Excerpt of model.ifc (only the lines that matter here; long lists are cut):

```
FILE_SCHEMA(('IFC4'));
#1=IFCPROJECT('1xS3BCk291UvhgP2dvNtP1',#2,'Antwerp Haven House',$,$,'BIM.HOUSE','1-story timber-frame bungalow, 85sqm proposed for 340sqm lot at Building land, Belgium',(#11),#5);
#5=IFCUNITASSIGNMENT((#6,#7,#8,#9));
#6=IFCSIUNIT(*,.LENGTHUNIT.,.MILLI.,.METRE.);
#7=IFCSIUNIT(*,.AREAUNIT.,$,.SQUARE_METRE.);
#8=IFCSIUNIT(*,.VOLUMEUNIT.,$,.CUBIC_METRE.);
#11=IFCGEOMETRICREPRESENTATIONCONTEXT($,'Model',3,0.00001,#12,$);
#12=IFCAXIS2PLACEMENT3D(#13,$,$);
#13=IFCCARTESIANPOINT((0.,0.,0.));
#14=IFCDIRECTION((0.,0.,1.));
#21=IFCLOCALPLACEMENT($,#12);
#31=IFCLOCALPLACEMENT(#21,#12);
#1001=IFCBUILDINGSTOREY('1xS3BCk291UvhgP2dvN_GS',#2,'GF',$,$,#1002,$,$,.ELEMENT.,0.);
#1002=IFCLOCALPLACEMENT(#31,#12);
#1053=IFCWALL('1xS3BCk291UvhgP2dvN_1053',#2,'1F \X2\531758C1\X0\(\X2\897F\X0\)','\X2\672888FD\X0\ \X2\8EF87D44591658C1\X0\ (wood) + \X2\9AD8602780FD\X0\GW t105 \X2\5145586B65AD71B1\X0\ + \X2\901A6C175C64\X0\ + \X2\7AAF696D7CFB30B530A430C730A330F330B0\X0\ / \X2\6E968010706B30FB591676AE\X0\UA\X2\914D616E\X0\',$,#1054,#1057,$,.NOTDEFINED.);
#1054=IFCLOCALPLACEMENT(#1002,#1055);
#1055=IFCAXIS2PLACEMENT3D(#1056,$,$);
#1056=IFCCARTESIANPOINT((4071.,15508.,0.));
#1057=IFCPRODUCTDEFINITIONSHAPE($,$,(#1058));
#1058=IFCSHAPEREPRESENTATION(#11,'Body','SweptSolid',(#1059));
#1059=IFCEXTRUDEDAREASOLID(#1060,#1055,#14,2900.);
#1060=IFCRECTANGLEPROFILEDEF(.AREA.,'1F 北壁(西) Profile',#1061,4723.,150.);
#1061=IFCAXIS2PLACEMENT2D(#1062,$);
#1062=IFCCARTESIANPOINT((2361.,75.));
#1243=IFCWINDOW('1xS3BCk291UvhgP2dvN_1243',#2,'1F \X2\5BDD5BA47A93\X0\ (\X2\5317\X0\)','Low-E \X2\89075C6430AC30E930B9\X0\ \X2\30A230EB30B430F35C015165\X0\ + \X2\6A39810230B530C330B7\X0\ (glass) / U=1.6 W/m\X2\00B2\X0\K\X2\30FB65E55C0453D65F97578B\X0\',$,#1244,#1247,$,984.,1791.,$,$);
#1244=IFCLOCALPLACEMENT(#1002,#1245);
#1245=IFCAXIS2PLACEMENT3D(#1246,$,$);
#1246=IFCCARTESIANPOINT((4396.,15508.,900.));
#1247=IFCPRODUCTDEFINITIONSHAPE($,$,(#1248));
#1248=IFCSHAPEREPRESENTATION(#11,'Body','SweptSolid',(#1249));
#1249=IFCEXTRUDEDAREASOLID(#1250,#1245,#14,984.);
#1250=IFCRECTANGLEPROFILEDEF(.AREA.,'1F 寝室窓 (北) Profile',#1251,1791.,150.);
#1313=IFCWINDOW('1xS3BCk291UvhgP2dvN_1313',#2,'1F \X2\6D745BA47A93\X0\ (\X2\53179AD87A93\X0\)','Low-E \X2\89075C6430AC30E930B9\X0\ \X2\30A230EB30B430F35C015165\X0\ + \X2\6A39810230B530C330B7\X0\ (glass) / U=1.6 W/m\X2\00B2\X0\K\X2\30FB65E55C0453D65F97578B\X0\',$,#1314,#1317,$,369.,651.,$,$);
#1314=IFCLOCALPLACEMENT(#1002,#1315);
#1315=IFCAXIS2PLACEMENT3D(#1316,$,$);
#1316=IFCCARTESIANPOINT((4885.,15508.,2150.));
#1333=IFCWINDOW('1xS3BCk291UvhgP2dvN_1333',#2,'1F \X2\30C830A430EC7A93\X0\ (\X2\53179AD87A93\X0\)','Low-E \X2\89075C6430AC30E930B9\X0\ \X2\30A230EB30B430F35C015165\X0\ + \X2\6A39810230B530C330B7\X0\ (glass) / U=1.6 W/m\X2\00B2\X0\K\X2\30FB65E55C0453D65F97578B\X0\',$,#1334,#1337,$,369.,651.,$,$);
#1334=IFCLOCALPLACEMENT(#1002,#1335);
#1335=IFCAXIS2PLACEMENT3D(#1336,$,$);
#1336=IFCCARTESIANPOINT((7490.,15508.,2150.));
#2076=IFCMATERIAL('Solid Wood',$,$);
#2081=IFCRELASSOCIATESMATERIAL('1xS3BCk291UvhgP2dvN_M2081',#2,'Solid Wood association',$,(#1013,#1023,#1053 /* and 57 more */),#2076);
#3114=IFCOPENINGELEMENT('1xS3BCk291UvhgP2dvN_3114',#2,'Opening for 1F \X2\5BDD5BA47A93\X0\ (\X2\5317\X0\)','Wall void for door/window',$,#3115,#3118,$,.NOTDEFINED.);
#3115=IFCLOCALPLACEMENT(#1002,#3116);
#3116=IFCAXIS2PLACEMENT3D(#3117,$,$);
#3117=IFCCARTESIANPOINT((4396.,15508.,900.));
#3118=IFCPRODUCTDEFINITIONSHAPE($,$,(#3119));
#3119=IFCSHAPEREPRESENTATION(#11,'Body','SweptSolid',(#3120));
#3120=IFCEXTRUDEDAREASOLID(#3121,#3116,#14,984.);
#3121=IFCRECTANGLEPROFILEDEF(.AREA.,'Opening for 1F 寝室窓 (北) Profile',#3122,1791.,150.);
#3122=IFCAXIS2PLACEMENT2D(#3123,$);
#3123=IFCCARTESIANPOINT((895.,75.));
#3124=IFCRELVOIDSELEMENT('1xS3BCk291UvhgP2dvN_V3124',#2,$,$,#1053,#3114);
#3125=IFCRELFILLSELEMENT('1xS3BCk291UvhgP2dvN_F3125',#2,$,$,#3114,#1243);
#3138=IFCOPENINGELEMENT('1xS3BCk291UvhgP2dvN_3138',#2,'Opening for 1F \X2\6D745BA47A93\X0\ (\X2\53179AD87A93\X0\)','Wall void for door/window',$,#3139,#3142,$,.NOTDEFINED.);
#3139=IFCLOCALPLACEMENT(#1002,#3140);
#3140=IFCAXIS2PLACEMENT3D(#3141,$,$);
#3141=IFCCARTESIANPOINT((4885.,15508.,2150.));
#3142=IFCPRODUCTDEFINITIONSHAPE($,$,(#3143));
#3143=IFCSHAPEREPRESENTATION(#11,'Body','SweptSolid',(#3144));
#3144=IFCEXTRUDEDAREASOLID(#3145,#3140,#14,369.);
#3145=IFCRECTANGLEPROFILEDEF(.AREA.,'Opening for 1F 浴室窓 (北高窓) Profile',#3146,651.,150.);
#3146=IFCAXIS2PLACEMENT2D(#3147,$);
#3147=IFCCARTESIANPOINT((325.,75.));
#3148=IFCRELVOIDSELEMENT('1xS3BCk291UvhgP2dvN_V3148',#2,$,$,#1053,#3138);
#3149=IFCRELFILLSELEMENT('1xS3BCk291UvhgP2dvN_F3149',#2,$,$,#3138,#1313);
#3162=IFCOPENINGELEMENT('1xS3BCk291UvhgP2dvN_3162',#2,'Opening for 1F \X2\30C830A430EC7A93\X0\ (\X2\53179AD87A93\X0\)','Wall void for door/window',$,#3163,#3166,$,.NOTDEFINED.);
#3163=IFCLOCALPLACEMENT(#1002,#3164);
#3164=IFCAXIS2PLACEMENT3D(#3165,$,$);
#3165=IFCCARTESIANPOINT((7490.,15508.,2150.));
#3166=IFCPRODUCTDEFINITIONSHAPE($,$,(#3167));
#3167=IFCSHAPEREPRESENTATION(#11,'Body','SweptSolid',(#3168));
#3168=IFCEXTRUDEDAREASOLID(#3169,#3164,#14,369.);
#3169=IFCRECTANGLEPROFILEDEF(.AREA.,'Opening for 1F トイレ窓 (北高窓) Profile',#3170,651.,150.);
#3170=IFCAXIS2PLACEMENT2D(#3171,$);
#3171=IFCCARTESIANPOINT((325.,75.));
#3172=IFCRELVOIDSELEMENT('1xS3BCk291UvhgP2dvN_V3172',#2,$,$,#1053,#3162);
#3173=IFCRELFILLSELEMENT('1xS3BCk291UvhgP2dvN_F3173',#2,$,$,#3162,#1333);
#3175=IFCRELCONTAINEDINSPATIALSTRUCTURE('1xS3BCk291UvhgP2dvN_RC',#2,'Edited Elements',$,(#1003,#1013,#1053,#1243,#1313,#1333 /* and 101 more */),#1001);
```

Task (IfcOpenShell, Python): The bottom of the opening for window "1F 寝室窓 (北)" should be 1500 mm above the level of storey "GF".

```python
import numpy as np
import ifcopenshell
import ifcopenshell.api.geometry
import ifcopenshell.geom
import ifcopenshell.util.element
import ifcopenshell.util.placement
import ifcopenshell.util.shape
import ifcopenshell.util.unit

model = ifcopenshell.open("model.ifc")
unit_scale = ifcopenshell.util.unit.calculate_unit_scale(model)

window = model.by_guid("1xS3BCk291UvhgP2dvN_1243")
opening = window.FillsVoids[0].RelatingOpeningElement
storey = ifcopenshell.util.element.get_container(window, ifc_class="IfcBuildingStorey")
level = ifcopenshell.util.placement.get_local_placement(storey.ObjectPlacement)[2, 3]

# The opening's origin need not be at the sill, so measure its lowest point.
shape = ifcopenshell.geom.create_shape(ifcopenshell.geom.settings(), opening)
bottom = ifcopenshell.util.shape.get_shape_bottom_elevation(shape, shape.geometry) / unit_scale
dz = level + 1500.0 - bottom

shift = np.array([0.0, 0.0, dz])
# The window is not placed relative to its opening, so move both.
for product in (opening, window):
    matrix = ifcopenshell.util.placement.get_local_placement(product.ObjectPlacement)
    matrix[:3, 3] += shift
    ifcopenshell.api.geometry.edit_object_placement(model, product=product, matrix=matrix, is_si=False)

print(f"moved by {dz * unit_scale:+.3f} m")

model.write("model_edited.ifc")
```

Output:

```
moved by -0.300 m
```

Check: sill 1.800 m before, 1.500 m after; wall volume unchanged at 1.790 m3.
